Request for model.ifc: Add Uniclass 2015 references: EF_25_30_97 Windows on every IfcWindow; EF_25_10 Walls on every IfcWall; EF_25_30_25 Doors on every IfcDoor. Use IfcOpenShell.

First a look at what the model holds.

```python
import ifcopenshell

model = ifcopenshell.open("model.ifc")
print(model.schema)
print("classifications:", [c.Name for c in model.by_type("IfcClassification")])
for ifc_class in ("IfcDoor", "IfcRoof", "IfcStair", "IfcWall", "IfcWindow"):
    print(ifc_class, len(model.by_type(ifc_class)))
```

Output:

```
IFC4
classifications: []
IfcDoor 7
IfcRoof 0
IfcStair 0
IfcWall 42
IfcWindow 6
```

```python
import ifcopenshell
import ifcopenshell.api.classification

model = ifcopenshell.open("model.ifc")

system = ifcopenshell.api.classification.add_classification(model, classification="Uniclass 2015")

codes = {
    "IfcWindow": ("EF_25_30_97", "Windows"),
    "IfcWall": ("EF_25_10", "Walls"),
    "IfcDoor": ("EF_25_30_25", "Doors"),
}
for ifc_class, (code, name) in codes.items():
    products = model.by_type(ifc_class)
    ifcopenshell.api.classification.add_reference(
        model, products=products, classification=system, identification=code, name=name
    )
    print(code, len(products))

model.write("model_v2.ifc")
```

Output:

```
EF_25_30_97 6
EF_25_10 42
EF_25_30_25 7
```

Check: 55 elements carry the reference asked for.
